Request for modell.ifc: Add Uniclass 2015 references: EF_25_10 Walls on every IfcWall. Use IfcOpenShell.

First a look at what the model holds.

```python
import ifcopenshell

model = ifcopenshell.open("modell.ifc")
print(model.schema)
print("classifications:", [c.Name for c in model.by_type("IfcClassification")])
for ifc_class in ("IfcDoor", "IfcRoof", "IfcStair", "IfcWall", "IfcWindow"):
    print(ifc_class, len(model.by_type(ifc_class)))
```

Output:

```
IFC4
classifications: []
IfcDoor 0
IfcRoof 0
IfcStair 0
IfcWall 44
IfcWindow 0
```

```python
import ifcopenshell
import ifcopenshell.api.classification

model = ifcopenshell.open("modell.ifc")

system = ifcopenshell.api.classification.add_classification(model, classification="Uniclass 2015")

codes = {
    "IfcWall": ("EF_25_10", "Walls"),
}
for ifc_class, (code, name) in codes.items():
    products = model.by_type(ifc_class)
    ifcopenshell.api.classification.add_reference(
        model, products=products, classification=system, identification=code, name=name
    )
    print(code, len(products))

model.write("modell_updated.ifc")
```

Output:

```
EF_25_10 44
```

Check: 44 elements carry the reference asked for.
